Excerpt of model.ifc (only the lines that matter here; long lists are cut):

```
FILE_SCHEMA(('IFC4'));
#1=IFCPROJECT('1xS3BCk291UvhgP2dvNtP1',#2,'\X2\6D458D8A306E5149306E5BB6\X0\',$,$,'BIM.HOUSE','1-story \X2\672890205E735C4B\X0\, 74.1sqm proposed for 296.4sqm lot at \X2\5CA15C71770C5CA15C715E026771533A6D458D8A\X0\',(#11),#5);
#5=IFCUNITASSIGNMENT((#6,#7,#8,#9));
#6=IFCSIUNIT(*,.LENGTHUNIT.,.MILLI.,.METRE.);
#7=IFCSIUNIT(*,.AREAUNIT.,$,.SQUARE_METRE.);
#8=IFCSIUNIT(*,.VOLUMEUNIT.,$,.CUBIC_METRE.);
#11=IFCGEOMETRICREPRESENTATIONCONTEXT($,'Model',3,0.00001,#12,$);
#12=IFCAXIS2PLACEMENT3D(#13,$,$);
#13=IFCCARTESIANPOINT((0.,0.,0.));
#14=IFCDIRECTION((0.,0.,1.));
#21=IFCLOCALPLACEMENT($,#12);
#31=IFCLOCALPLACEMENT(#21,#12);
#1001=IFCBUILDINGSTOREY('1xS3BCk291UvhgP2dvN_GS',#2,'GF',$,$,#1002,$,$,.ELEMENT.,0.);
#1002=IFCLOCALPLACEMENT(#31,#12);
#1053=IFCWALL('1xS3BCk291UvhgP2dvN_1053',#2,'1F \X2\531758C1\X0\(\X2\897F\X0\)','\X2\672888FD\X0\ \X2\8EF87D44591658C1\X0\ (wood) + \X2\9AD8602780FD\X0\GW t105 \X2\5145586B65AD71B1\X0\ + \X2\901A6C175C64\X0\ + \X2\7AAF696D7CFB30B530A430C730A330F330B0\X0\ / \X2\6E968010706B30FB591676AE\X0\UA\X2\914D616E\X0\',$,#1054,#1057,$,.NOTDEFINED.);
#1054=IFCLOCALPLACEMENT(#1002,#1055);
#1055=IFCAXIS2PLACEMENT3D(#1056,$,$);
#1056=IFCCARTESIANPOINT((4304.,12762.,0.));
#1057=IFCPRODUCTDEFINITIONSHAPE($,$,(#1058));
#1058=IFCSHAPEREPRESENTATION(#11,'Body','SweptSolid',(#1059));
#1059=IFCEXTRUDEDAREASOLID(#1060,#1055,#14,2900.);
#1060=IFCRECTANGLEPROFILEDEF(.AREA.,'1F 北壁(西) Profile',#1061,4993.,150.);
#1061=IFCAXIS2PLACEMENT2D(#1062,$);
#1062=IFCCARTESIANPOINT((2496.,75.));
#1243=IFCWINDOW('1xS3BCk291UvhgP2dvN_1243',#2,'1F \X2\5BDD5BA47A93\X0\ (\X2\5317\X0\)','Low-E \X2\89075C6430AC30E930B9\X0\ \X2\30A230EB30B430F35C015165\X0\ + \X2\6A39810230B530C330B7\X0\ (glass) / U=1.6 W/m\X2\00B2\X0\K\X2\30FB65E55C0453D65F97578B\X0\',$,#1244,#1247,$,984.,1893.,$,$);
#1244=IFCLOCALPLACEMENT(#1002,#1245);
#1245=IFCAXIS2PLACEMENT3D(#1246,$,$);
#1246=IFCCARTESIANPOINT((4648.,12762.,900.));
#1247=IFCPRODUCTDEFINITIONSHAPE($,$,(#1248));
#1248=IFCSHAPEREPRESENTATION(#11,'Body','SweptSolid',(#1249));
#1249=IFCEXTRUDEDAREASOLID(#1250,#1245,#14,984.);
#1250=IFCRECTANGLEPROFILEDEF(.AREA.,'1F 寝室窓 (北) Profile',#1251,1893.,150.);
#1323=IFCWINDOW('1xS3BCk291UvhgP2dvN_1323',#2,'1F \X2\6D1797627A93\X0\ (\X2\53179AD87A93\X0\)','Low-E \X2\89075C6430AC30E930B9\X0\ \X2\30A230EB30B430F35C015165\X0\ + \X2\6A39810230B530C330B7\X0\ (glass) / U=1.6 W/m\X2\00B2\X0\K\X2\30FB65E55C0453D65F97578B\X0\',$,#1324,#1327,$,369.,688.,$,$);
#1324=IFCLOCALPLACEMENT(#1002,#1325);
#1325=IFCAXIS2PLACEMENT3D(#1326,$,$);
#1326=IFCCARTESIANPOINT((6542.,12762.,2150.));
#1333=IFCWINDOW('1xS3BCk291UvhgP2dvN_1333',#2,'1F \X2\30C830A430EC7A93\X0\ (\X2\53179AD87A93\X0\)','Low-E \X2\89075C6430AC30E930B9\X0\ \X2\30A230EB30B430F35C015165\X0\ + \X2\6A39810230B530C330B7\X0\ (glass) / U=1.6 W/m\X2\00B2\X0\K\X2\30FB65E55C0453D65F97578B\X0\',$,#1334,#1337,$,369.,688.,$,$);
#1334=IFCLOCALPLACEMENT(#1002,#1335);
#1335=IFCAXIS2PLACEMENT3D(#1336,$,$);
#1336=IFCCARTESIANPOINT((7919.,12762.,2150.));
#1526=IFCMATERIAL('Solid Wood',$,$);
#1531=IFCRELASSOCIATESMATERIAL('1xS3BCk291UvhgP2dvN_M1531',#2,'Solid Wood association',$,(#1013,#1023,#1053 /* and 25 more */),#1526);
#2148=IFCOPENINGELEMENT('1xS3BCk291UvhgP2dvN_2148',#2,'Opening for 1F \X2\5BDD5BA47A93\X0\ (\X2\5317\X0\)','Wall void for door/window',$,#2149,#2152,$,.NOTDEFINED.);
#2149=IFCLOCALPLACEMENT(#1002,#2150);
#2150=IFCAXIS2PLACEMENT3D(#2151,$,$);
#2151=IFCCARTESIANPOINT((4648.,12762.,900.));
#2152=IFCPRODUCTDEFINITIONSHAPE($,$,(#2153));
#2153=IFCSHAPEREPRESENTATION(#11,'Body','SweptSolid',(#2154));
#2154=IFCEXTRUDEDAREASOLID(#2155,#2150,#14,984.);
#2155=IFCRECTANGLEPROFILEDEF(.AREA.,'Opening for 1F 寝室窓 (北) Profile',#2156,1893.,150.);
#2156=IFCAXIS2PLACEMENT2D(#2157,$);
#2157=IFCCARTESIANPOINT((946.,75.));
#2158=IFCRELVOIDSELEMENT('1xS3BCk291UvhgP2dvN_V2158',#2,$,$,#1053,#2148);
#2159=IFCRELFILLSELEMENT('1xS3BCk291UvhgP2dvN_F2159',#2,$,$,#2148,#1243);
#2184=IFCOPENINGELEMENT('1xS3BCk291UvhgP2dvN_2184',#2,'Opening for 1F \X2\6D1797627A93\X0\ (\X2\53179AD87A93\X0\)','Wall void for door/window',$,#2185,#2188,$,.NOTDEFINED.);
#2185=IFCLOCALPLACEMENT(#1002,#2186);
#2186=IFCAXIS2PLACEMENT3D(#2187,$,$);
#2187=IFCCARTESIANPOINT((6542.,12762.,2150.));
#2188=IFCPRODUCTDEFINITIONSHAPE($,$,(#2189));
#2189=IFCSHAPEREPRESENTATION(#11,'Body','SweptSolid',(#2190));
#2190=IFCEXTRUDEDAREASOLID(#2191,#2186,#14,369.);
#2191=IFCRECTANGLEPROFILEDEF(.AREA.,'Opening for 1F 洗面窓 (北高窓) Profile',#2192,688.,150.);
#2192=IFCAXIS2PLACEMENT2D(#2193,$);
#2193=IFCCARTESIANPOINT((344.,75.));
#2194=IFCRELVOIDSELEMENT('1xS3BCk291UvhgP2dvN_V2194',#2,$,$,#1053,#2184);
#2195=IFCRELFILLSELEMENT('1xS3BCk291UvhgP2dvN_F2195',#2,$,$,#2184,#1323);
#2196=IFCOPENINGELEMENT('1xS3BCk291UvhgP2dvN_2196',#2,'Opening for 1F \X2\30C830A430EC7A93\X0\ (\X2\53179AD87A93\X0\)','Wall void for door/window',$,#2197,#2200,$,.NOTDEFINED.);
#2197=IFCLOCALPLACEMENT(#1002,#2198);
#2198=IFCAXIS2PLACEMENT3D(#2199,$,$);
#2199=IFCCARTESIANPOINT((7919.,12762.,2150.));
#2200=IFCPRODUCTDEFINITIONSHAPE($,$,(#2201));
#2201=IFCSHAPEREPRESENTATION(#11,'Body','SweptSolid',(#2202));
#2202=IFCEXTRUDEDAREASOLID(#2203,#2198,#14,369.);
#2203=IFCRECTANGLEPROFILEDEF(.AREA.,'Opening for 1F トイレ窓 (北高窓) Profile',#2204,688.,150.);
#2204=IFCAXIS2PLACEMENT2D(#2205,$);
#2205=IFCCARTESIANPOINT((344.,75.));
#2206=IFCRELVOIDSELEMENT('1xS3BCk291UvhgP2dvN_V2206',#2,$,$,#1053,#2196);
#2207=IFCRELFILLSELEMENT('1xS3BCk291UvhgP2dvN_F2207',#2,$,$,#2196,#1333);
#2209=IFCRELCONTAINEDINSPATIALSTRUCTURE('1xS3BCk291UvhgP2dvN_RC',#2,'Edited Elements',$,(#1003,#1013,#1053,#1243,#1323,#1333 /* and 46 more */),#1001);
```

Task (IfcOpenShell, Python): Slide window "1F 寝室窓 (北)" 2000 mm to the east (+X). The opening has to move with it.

```python
import ifcopenshell
import ifcopenshell.api.geometry
import ifcopenshell.util.placement

model = ifcopenshell.open("model.ifc")

window = model.by_guid("1xS3BCk291UvhgP2dvN_1243")
opening = window.FillsVoids[0].RelatingOpeningElement
wall = opening.VoidsElements[0].RelatingBuildingElement

wall_matrix = ifcopenshell.util.placement.get_local_placement(wall.ObjectPlacement)
shift = wall_matrix[:3, 0] * 2000.0
before = ifcopenshell.util.placement.get_local_placement(window.ObjectPlacement)[:3, 3].copy()

# The window is not placed relative to its opening, so move both.
for product in (opening, window):
    matrix = ifcopenshell.util.placement.get_local_placement(product.ObjectPlacement)
    matrix[:3, 3] += shift
    ifcopenshell.api.geometry.edit_object_placement(model, product=product, matrix=matrix, is_si=False)

after = ifcopenshell.util.placement.get_local_placement(window.ObjectPlacement)[:3, 3]
print("window moved by", (after - before).round(3) + 0.0)

model.write("model-out.ifc")
```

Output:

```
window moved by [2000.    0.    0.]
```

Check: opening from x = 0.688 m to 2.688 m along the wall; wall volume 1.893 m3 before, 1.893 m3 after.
